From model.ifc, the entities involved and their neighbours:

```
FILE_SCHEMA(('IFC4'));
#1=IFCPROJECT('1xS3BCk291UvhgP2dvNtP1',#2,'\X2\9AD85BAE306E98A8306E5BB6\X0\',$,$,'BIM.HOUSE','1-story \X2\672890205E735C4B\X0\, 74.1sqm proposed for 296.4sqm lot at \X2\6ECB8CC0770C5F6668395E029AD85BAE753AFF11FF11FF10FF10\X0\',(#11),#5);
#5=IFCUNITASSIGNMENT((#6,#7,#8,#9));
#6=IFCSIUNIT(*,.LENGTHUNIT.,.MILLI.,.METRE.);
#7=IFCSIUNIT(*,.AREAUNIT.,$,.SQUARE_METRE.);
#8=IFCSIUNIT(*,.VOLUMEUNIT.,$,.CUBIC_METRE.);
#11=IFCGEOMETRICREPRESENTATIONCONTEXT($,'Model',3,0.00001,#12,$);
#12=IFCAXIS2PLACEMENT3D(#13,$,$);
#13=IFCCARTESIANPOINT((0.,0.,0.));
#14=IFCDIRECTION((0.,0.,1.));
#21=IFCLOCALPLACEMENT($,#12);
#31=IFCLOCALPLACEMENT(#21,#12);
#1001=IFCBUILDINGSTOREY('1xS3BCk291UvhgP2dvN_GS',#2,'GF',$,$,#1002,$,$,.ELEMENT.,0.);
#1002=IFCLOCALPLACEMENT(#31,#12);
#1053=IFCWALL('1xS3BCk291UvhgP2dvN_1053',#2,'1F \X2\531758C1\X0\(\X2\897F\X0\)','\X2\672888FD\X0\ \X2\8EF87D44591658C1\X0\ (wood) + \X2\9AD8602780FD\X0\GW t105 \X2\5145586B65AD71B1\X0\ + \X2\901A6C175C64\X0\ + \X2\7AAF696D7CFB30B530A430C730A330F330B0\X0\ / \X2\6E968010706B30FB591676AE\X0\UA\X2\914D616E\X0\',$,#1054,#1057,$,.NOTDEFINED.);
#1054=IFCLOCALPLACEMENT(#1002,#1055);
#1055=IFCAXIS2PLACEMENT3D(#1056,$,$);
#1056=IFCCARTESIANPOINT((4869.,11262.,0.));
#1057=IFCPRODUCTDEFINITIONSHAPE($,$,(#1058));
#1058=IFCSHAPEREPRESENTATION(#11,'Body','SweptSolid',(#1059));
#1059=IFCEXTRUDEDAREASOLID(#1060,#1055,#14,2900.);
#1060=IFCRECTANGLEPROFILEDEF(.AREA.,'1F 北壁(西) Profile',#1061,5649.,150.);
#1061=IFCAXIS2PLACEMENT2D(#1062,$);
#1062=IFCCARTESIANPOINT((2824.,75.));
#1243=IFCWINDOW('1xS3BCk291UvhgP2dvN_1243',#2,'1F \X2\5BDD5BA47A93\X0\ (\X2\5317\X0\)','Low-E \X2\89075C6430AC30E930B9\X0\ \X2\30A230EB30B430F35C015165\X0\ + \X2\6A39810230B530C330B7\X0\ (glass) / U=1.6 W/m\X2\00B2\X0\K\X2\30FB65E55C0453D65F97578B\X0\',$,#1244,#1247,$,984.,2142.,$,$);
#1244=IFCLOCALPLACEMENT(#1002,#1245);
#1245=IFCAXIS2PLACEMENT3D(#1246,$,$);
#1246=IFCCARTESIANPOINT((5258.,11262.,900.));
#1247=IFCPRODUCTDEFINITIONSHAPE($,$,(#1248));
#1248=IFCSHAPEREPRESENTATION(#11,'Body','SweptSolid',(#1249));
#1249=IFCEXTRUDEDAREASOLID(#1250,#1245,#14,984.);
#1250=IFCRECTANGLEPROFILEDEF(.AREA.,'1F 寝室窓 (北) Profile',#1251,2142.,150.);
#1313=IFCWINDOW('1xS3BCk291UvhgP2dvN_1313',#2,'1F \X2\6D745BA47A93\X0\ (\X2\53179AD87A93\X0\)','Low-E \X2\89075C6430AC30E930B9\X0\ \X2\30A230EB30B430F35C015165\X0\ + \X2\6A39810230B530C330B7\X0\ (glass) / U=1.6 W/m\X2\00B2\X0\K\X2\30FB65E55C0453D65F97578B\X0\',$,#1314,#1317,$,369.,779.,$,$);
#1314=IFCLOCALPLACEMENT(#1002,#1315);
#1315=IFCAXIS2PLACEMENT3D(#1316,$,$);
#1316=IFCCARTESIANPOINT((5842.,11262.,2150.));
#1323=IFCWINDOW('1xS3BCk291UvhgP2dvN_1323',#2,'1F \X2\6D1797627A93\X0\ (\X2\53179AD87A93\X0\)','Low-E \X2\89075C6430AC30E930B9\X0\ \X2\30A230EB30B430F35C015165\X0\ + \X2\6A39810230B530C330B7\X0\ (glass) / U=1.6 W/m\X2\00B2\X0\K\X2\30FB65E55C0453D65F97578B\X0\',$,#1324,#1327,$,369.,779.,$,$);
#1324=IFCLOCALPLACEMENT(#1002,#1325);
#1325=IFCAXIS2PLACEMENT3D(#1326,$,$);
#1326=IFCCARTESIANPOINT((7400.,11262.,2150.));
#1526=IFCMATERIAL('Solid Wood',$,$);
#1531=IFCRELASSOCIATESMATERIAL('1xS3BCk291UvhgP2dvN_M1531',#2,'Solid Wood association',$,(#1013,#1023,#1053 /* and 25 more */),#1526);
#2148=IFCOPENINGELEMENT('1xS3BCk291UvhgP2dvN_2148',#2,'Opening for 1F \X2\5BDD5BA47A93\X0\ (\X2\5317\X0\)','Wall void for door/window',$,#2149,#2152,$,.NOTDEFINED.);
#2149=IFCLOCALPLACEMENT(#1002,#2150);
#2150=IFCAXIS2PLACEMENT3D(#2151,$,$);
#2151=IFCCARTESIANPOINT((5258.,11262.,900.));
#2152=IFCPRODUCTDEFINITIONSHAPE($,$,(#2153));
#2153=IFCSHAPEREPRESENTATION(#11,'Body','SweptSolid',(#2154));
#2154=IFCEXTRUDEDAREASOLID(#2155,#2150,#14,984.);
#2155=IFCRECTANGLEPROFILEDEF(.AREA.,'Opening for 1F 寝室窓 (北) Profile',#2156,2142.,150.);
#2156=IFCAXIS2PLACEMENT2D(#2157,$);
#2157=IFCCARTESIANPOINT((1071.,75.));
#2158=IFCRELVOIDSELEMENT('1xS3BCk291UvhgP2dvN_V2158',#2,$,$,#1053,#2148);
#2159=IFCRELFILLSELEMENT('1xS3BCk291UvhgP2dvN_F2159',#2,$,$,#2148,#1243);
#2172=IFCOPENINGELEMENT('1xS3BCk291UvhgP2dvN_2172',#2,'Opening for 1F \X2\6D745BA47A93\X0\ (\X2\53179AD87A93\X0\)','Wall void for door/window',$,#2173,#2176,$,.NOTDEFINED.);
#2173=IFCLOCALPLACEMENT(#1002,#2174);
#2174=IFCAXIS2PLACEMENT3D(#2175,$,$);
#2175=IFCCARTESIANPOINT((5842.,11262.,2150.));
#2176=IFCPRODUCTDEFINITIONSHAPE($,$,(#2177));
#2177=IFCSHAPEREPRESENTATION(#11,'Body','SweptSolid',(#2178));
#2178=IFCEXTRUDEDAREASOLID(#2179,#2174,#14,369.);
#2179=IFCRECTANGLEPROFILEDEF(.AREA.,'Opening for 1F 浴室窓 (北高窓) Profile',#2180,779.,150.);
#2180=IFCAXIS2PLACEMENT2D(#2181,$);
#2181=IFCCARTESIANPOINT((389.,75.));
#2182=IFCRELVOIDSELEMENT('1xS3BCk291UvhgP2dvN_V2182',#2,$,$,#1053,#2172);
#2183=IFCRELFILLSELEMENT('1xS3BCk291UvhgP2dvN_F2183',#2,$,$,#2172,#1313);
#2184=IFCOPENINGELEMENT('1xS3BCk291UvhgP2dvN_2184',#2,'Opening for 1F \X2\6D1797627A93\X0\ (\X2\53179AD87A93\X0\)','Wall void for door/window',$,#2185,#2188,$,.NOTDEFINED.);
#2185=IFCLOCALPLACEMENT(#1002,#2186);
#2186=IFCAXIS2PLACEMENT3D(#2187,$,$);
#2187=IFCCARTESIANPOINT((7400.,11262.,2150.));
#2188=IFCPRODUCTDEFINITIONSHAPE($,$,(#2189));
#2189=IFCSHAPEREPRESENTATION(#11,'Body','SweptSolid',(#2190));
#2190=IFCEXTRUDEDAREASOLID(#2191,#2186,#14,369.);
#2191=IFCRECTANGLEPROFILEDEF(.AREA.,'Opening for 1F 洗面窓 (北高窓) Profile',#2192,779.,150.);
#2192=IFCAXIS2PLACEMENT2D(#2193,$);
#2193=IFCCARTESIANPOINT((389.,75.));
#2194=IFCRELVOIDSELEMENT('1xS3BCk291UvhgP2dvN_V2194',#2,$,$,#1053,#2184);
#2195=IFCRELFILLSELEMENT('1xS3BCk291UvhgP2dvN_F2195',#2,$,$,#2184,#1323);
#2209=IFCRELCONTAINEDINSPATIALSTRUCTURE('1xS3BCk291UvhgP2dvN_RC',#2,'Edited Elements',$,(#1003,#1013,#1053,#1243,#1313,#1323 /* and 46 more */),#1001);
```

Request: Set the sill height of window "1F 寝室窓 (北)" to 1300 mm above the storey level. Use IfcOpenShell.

```python
import numpy as np
import ifcopenshell
import ifcopenshell.api.geometry
import ifcopenshell.geom
import ifcopenshell.util.element
import ifcopenshell.util.placement
import ifcopenshell.util.shape
import ifcopenshell.util.unit

model = ifcopenshell.open("model.ifc")
unit_scale = ifcopenshell.util.unit.calculate_unit_scale(model)

window = model.by_guid("1xS3BCk291UvhgP2dvN_1243")
opening = window.FillsVoids[0].RelatingOpeningElement
storey = ifcopenshell.util.element.get_container(window, ifc_class="IfcBuildingStorey")
level = ifcopenshell.util.placement.get_local_placement(storey.ObjectPlacement)[2, 3]

# The opening's origin need not be at the sill, so measure its lowest point.
shape = ifcopenshell.geom.create_shape(ifcopenshell.geom.settings(), opening)
bottom = ifcopenshell.util.shape.get_shape_bottom_elevation(shape, shape.geometry) / unit_scale
dz = level + 1.3 / unit_scale - bottom

shift = np.array([0.0, 0.0, dz])
# The window is not placed relative to its opening, so move both.
for product in (opening, window):
    matrix = ifcopenshell.util.placement.get_local_placement(product.ObjectPlacement)
    matrix[:3, 3] += shift
    ifcopenshell.api.geometry.edit_object_placement(model, product=product, matrix=matrix, is_si=False)

print(f"moved by {dz * unit_scale:+.3f} m")

model.write("model_edited.ifc")
```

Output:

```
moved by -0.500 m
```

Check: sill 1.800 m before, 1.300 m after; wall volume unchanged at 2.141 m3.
